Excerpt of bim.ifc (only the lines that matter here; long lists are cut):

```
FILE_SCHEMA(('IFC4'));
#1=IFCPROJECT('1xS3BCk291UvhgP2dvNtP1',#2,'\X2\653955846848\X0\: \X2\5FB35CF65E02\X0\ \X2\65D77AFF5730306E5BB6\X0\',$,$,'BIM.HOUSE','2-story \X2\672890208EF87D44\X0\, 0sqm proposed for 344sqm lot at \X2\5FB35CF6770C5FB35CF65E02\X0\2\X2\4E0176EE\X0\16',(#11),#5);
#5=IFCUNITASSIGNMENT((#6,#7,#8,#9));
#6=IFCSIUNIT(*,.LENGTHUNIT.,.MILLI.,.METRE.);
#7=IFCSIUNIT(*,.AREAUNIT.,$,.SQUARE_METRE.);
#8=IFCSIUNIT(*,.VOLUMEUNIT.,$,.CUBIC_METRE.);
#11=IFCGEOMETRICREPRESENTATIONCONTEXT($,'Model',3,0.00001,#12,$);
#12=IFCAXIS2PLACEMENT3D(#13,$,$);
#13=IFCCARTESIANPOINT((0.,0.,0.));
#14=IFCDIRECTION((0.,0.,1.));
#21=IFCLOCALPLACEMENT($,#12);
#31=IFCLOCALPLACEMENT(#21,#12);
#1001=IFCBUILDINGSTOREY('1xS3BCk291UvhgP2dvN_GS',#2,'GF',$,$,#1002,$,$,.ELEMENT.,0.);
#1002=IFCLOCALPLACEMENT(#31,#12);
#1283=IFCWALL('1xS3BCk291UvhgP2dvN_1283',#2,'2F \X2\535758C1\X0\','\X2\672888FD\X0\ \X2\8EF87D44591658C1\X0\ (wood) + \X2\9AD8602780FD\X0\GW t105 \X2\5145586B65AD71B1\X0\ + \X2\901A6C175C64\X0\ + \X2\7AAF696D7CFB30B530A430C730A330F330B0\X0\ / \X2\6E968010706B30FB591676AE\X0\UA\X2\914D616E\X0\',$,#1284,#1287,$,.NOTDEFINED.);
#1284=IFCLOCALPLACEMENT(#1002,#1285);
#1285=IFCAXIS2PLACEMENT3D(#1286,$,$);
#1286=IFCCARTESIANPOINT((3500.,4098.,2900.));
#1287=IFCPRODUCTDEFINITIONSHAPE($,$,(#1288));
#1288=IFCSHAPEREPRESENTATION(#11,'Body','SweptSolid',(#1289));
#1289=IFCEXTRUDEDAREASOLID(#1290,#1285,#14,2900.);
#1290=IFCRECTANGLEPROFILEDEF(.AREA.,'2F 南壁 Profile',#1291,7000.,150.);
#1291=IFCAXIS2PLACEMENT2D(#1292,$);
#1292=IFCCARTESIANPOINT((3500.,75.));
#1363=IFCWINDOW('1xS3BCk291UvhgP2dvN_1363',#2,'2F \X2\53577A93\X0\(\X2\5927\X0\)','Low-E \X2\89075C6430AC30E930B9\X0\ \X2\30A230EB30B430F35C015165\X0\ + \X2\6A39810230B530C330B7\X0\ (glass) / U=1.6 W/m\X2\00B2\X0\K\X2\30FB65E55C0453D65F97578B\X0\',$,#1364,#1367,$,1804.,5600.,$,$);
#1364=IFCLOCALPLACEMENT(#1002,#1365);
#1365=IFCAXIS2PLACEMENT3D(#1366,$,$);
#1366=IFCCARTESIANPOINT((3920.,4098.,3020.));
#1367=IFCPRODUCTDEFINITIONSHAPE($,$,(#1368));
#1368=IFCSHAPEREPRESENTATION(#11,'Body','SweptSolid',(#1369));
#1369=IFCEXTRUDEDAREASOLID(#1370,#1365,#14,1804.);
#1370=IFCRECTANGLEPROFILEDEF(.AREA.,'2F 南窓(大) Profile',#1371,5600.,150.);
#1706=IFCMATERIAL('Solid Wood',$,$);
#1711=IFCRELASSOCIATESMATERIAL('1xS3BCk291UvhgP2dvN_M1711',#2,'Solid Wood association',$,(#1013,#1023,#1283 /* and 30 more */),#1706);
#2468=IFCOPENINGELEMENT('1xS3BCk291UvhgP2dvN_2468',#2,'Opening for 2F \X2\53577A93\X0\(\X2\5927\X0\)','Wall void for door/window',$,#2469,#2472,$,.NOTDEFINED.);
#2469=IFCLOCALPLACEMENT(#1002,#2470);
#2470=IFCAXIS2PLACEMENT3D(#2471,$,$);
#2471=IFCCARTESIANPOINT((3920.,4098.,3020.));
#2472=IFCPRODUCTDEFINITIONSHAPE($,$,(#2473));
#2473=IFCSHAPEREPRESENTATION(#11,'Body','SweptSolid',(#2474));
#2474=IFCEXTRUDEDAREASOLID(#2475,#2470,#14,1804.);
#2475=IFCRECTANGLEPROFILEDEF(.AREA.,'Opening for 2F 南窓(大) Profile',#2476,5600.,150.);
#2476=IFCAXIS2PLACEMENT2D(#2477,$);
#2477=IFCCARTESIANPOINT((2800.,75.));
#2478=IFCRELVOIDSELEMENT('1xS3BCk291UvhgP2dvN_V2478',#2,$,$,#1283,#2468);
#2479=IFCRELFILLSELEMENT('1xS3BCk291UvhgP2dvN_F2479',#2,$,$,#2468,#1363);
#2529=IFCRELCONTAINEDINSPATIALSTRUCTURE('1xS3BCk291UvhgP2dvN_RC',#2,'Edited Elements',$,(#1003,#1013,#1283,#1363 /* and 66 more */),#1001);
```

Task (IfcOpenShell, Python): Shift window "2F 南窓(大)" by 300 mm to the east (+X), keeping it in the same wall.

```python
import ifcopenshell
import ifcopenshell.api.geometry
import ifcopenshell.util.placement
import ifcopenshell.util.unit

model = ifcopenshell.open("bim.ifc")
unit_scale = ifcopenshell.util.unit.calculate_unit_scale(model)

window = model.by_guid("1xS3BCk291UvhgP2dvN_1363")
opening = window.FillsVoids[0].RelatingOpeningElement
wall = opening.VoidsElements[0].RelatingBuildingElement

wall_matrix = ifcopenshell.util.placement.get_local_placement(wall.ObjectPlacement)
shift = wall_matrix[:3, 0] * 0.3 / unit_scale
before = ifcopenshell.util.placement.get_local_placement(window.ObjectPlacement)[:3, 3].copy()

# The window is not placed relative to its opening, so move both.
for product in (opening, window):
    matrix = ifcopenshell.util.placement.get_local_placement(product.ObjectPlacement)
    matrix[:3, 3] += shift
    ifcopenshell.api.geometry.edit_object_placement(model, product=product, matrix=matrix, is_si=False)

after = ifcopenshell.util.placement.get_local_placement(window.ObjectPlacement)[:3, 3]
print("window moved by", (after - before).round(3) + 0.0)

model.write("bim-out.ifc")
```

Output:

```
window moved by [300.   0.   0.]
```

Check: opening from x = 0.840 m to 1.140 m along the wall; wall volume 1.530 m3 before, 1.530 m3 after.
